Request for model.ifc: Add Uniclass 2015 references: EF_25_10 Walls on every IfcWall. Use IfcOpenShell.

First a look at what the model holds.

```python
import ifcopenshell

model = ifcopenshell.open("model.ifc")
print(model.schema)
print("classifications:", [c.Name for c in model.by_type("IfcClassification")])
for ifc_class in ("IfcDoor", "IfcRoof", "IfcStair", "IfcWall", "IfcWindow"):
    print(ifc_class, len(model.by_type(ifc_class)))
```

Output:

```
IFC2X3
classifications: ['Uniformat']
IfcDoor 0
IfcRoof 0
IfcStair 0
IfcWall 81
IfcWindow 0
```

```python
import ifcopenshell
import ifcopenshell.api.classification

model = ifcopenshell.open("model.ifc")

# IFC2X3 requires Source and Edition and has no link from the project to the system.
system = model.create_entity("IfcClassification", Source="NBS", Edition="2015", Name="Uniclass 2015")

codes = {
    "IfcWall": ("EF_25_10", "Walls"),
}
for ifc_class, (code, name) in codes.items():
    products = model.by_type(ifc_class)
    ifcopenshell.api.classification.add_reference(
        model, products=products, classification=system, identification=code, name=name
    )
    print(code, len(products))

model.write("model_edited.ifc")
```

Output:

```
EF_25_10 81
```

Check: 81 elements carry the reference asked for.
